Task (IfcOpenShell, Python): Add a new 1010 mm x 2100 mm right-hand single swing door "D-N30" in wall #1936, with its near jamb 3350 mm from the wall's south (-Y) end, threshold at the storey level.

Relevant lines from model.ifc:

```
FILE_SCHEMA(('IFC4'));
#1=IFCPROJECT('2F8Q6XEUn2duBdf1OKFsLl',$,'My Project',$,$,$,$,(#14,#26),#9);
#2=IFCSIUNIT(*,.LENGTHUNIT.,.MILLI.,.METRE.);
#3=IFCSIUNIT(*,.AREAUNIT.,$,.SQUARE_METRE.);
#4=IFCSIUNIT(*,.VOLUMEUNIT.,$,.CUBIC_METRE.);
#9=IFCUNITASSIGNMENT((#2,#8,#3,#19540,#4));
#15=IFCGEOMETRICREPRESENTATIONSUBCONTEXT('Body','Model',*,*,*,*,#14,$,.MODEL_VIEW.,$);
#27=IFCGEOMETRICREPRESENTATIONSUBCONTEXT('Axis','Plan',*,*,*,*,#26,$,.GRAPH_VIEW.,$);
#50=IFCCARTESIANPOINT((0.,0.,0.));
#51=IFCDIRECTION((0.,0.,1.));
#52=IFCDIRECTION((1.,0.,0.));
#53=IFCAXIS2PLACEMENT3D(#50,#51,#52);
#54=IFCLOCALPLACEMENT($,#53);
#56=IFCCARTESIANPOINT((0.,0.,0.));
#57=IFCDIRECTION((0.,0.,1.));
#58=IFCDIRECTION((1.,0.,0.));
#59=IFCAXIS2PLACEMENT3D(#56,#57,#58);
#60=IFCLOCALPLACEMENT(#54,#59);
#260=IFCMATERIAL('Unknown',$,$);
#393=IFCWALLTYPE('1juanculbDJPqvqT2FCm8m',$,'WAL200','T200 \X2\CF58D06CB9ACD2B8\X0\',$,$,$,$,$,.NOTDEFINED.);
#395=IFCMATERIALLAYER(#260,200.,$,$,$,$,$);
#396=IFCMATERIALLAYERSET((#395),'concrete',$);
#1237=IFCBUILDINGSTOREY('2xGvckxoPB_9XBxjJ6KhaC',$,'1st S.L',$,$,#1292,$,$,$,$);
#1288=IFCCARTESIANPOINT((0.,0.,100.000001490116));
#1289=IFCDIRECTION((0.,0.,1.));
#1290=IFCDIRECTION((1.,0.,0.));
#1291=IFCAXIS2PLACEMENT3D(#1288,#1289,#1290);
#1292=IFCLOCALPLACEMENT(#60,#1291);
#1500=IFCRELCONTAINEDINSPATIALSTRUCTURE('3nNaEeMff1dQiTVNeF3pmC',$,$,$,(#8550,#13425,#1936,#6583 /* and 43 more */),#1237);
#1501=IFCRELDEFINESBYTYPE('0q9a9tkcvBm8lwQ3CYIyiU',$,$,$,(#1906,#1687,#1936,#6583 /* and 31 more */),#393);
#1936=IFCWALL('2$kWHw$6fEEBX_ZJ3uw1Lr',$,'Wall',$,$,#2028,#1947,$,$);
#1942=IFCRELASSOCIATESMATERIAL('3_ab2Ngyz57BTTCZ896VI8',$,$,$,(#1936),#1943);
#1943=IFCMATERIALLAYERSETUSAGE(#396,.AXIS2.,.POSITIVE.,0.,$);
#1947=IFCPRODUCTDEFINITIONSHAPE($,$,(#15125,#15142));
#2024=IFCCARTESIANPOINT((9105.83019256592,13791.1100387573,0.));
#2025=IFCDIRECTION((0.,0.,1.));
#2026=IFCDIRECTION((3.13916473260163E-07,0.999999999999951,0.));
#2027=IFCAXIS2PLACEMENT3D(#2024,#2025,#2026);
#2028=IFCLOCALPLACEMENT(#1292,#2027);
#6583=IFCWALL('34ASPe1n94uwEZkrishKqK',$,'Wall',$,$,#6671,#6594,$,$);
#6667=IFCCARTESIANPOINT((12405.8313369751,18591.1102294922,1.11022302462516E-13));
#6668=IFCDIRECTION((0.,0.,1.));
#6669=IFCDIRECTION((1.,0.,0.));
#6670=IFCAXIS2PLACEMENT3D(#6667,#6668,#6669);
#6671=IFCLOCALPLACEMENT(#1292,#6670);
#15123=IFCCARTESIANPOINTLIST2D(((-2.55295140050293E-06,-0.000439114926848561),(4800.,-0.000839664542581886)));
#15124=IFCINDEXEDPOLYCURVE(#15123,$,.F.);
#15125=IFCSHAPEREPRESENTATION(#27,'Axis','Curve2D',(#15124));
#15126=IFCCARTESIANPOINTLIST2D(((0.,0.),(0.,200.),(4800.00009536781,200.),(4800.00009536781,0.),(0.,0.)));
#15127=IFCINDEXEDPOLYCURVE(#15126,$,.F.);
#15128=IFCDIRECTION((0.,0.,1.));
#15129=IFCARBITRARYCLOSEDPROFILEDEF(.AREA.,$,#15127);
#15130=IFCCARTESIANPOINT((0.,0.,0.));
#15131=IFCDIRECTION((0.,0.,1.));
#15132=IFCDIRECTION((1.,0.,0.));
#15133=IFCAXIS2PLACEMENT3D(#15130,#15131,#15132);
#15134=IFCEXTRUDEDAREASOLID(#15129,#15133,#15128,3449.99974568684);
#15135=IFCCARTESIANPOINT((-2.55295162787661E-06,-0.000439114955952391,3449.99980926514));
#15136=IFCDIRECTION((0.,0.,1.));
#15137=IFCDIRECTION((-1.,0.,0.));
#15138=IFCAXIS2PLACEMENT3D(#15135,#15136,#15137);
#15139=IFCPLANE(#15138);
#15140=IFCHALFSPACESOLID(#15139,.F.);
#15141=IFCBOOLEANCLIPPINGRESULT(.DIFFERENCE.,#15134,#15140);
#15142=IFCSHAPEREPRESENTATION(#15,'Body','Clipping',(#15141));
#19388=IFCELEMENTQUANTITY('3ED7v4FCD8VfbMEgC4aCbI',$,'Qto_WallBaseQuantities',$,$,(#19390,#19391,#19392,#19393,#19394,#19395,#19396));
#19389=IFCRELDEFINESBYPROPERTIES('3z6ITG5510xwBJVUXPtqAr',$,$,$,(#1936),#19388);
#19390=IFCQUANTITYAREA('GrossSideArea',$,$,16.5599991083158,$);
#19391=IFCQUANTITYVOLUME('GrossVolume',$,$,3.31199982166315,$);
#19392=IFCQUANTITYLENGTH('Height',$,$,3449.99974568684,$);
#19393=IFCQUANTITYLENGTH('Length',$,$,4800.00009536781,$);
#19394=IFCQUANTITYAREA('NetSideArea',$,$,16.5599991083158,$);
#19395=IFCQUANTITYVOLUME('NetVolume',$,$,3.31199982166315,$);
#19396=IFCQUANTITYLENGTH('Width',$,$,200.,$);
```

```python
import numpy as np
import ifcopenshell
import ifcopenshell.api.feature
import ifcopenshell.api.geometry
import ifcopenshell.api.pset
import ifcopenshell.api.root
import ifcopenshell.api.spatial
import ifcopenshell.geom
import ifcopenshell.util.element
import ifcopenshell.util.placement
import ifcopenshell.util.representation
import ifcopenshell.util.shape
import ifcopenshell.util.unit

model = ifcopenshell.open("model.ifc")
unit_scale = ifcopenshell.util.unit.calculate_unit_scale(model)
area_scale = ifcopenshell.util.unit.calculate_unit_scale(model, "AREAUNIT")
volume_scale = ifcopenshell.util.unit.calculate_unit_scale(model, "VOLUMEUNIT")
settings = ifcopenshell.geom.settings()


def volume(element):
    """Net volume in cubic metres, openings subtracted."""
    shape = ifcopenshell.geom.create_shape(settings, element)
    return ifcopenshell.util.shape.get_volume(shape.geometry)


wall = model.by_guid("2$kWHw$6fEEBX_ZJ3uw1Lr")
storey = ifcopenshell.util.element.get_container(wall, ifc_class="IfcBuildingStorey")
context = ifcopenshell.util.representation.get_context(model, "Model", "Body", "MODEL_VIEW")
before = volume(wall)

width, height, from_end, sill = 1.01, 2.1, 3.35, 0.0  # metres

# The wall runs along its own X axis, and the end named is its -X end.
wall_shape = ifcopenshell.geom.create_shape(settings, wall)
x, y, z = ifcopenshell.util.shape.get_vertices(wall_shape.geometry).T
start = x.min() + from_end
face, thickness = float(y.min()), float(y.max() - y.min())
wall_matrix = ifcopenshell.util.placement.get_local_placement(wall.ObjectPlacement)
level = ifcopenshell.util.placement.get_local_placement(storey.ObjectPlacement)[2, 3]


def in_wall(x, y):
    """Placement at x, y metres in the wall's axes, at sill height."""
    matrix = wall_matrix.copy()
    matrix[:, 3] = wall_matrix @ np.array([x / unit_scale, y / unit_scale, 0.0, 1.0])
    matrix[2, 3] = level + sill / unit_scale
    return matrix


# Opening: a box that overshoots both wall faces by 50 mm.
opening = ifcopenshell.api.root.create_entity(model, ifc_class="IfcOpeningElement", predefined_type="OPENING")
box = ifcopenshell.api.geometry.add_wall_representation(
    model, context=context, length=width, height=height, thickness=thickness + 0.1
)
ifcopenshell.api.geometry.assign_representation(model, product=opening, representation=box)
ifcopenshell.api.geometry.edit_object_placement(model, product=opening, matrix=in_wall(start, face - 0.05), is_si=False)
ifcopenshell.api.feature.add_feature(model, feature=opening, element=wall)

door = ifcopenshell.api.root.create_entity(model, ifc_class="IfcDoor", name="D-N30", predefined_type="DOOR")
door.OverallWidth, door.OverallHeight = width / unit_scale, height / unit_scale
door.OperationType = "SINGLE_SWING_RIGHT"
body = ifcopenshell.api.geometry.add_door_representation(
    model,
    context=context,
    overall_width=door.OverallWidth,
    overall_height=door.OverallHeight,
    operation_type="SINGLE_SWING_RIGHT",
    lining_properties={"LiningDepth": thickness / unit_scale, "ThresholdDepth": thickness / unit_scale},
)
ifcopenshell.api.geometry.assign_representation(model, product=door, representation=body)
ifcopenshell.api.spatial.assign_container(model, products=[door], relating_structure=storey)
ifcopenshell.api.feature.add_filling(model, opening=opening, element=door)

# The lining spans the wall, so the door starts at the wall face.
ifcopenshell.api.geometry.edit_object_placement(model, product=door, matrix=in_wall(start, face), is_si=False)

after = volume(wall)

# Update the wall's stored quantities.
qto = model.by_id(ifcopenshell.util.element.get_pset(wall, "Qto_WallBaseQuantities", should_inherit=False)["id"])
ifcopenshell.api.pset.edit_qto(model, qto=qto, properties={
    "NetSideArea": after / thickness / area_scale,
    "NetVolume": after / volume_scale,
})

print(f"wall volume {before:.3f} -> {after:.3f} m3")

model.write("model-out.ifc")
```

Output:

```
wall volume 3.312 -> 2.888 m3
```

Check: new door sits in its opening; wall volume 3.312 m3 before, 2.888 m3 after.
